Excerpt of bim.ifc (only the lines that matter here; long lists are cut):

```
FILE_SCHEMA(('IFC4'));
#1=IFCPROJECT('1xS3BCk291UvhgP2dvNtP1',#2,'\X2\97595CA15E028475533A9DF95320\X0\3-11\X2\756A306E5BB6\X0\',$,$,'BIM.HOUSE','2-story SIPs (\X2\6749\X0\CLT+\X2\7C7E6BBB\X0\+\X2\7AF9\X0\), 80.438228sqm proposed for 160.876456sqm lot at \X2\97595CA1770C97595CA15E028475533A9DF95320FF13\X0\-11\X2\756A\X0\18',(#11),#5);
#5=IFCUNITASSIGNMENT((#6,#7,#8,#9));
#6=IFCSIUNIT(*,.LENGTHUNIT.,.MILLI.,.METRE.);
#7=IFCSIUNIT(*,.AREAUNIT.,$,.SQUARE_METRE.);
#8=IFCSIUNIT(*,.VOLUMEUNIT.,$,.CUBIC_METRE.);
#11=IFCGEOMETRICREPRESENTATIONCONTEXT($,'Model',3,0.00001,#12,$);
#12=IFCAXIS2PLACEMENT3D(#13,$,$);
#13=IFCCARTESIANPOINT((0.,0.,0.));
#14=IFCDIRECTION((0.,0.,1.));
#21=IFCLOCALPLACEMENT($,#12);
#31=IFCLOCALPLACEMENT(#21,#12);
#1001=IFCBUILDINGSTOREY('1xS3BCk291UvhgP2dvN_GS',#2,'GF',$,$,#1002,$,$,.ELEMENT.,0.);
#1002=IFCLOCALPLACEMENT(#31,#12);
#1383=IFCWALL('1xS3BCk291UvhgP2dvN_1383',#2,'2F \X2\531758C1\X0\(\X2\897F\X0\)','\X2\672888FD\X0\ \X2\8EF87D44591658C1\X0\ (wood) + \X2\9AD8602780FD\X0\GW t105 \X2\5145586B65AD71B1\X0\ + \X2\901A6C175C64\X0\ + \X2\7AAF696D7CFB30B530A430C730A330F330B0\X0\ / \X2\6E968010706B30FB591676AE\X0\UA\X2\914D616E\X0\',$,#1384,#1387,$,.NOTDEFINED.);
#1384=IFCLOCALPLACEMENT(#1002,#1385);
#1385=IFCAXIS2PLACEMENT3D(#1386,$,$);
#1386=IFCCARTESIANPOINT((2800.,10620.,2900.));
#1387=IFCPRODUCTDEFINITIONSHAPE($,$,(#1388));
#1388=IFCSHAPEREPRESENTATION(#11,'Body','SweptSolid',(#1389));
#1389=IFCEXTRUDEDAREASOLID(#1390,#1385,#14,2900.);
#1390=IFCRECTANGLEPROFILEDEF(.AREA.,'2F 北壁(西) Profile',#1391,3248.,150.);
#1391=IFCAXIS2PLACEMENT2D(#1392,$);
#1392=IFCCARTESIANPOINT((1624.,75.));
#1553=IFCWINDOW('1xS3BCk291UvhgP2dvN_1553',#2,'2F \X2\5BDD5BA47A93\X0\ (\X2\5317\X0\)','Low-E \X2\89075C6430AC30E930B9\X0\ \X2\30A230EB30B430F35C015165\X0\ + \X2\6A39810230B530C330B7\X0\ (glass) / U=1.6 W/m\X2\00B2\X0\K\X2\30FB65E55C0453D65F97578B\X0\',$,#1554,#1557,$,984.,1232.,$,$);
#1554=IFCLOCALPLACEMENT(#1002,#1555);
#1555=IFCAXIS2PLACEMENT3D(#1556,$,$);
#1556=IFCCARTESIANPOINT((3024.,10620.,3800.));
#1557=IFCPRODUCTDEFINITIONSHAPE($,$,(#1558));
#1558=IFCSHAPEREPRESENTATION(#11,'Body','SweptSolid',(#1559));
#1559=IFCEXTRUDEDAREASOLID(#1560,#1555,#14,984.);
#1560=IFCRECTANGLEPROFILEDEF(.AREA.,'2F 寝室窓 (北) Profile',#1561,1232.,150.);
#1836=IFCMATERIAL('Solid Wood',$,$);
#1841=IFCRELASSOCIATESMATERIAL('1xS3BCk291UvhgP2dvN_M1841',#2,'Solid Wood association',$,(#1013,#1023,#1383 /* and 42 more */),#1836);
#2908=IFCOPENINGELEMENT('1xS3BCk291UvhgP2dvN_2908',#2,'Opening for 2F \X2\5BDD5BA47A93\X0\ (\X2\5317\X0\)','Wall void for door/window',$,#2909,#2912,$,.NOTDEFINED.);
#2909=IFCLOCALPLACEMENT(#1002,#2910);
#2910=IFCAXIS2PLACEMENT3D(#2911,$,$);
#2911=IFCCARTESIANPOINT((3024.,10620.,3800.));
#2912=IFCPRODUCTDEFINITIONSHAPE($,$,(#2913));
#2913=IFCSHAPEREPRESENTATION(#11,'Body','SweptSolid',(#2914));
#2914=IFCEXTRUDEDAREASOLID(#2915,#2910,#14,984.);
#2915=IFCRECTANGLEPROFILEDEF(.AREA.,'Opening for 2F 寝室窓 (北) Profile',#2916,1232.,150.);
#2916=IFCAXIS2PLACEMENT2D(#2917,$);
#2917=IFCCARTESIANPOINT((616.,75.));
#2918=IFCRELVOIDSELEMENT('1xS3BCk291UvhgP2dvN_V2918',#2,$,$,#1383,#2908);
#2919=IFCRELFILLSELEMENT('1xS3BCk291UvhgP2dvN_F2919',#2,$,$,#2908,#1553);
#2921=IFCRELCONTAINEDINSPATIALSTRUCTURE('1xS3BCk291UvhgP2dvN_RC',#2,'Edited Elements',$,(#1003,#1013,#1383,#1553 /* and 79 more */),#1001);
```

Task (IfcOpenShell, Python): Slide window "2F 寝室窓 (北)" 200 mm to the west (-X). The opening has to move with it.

```python
import ifcopenshell
import ifcopenshell.api.geometry
import ifcopenshell.util.placement

model = ifcopenshell.open("bim.ifc")

window = model.by_id(1553)
opening = window.FillsVoids[0].RelatingOpeningElement
wall = opening.VoidsElements[0].RelatingBuildingElement

wall_matrix = ifcopenshell.util.placement.get_local_placement(wall.ObjectPlacement)
shift = wall_matrix[:3, 0] * -200.0
before = ifcopenshell.util.placement.get_local_placement(window.ObjectPlacement)[:3, 3].copy()

# The window is not placed relative to its opening, so move both.
for product in (opening, window):
    matrix = ifcopenshell.util.placement.get_local_placement(product.ObjectPlacement)
    matrix[:3, 3] += shift
    ifcopenshell.api.geometry.edit_object_placement(model, product=product, matrix=matrix, is_si=False)

after = ifcopenshell.util.placement.get_local_placement(window.ObjectPlacement)[:3, 3]
print("window moved by", (after - before).round(3) + 0.0)

model.write("bim_edited.ifc")
```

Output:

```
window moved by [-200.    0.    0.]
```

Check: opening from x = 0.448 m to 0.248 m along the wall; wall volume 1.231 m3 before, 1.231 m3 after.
